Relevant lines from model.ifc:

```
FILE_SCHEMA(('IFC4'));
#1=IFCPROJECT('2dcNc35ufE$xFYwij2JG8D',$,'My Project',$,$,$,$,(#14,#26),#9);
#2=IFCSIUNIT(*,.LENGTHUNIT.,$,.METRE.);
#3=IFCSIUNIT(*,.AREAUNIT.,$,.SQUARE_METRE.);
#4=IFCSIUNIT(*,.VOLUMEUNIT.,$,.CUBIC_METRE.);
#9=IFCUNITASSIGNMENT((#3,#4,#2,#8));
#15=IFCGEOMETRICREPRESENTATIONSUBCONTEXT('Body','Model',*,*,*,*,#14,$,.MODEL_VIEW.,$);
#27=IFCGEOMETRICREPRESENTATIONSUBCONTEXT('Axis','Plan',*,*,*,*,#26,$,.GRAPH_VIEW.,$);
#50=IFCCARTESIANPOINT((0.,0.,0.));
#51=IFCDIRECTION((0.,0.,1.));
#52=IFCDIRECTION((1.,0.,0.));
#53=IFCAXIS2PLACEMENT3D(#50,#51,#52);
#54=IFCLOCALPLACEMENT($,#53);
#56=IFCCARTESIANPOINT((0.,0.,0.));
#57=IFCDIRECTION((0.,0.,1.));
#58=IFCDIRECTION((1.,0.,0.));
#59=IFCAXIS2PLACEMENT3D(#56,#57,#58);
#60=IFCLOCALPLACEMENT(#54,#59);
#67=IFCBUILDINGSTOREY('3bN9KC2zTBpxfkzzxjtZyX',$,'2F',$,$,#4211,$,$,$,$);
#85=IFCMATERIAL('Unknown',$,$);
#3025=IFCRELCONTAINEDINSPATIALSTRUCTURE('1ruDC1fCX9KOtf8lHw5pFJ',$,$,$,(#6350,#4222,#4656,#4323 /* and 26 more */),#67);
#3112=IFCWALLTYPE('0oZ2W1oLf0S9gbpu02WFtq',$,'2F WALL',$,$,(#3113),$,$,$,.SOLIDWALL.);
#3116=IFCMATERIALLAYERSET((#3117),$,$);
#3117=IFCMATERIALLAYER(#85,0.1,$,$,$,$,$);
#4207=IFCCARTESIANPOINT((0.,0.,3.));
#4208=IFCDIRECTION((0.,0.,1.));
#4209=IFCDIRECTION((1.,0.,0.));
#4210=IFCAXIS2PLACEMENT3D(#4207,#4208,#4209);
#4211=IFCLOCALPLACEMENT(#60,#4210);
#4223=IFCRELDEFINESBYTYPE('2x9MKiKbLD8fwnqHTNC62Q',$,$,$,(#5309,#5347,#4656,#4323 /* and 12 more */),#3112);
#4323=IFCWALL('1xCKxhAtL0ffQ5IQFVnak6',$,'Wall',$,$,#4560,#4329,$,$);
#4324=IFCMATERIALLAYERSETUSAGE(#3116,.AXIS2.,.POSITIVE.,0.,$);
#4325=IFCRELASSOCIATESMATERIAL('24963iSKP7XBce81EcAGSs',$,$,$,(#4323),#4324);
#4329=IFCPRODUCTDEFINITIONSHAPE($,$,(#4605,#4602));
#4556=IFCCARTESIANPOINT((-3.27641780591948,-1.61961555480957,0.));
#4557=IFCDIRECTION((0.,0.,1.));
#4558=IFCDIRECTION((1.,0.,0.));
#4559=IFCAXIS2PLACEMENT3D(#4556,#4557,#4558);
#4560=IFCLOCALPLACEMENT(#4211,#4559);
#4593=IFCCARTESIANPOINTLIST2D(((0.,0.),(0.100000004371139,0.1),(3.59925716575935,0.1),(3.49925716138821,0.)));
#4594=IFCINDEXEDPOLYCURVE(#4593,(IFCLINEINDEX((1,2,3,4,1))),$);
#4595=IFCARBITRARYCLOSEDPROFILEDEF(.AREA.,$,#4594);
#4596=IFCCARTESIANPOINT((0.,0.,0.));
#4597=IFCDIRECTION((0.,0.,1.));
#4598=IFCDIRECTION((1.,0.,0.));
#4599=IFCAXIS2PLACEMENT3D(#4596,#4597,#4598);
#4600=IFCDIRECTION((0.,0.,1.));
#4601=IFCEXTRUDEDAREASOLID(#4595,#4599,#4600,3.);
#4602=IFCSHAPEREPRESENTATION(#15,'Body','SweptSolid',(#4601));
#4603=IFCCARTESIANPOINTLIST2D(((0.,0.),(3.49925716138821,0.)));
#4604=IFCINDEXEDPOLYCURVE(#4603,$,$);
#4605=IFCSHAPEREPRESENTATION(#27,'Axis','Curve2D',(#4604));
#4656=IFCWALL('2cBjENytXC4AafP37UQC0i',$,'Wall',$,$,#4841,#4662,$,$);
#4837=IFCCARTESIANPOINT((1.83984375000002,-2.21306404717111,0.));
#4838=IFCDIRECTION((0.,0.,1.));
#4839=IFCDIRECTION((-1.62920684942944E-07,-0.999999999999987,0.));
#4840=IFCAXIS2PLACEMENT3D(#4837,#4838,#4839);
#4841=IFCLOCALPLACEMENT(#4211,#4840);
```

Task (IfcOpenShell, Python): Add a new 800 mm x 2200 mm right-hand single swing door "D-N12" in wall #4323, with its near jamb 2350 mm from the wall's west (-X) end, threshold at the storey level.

```python
import numpy as np
import ifcopenshell
import ifcopenshell.api.feature
import ifcopenshell.api.geometry
import ifcopenshell.api.root
import ifcopenshell.api.spatial
import ifcopenshell.geom
import ifcopenshell.util.element
import ifcopenshell.util.placement
import ifcopenshell.util.representation
import ifcopenshell.util.shape
import ifcopenshell.util.unit

model = ifcopenshell.open("model.ifc")
unit_scale = ifcopenshell.util.unit.calculate_unit_scale(model)
settings = ifcopenshell.geom.settings()


def volume(element):
    """Net volume in cubic metres, openings subtracted."""
    shape = ifcopenshell.geom.create_shape(settings, element)
    return ifcopenshell.util.shape.get_volume(shape.geometry)


wall = model.by_guid("1xCKxhAtL0ffQ5IQFVnak6")
storey = ifcopenshell.util.element.get_container(wall, ifc_class="IfcBuildingStorey")
context = ifcopenshell.util.representation.get_context(model, "Model", "Body", "MODEL_VIEW")
before = volume(wall)

width, height, from_end, sill = 0.8, 2.2, 2.35, 0.0  # metres

# The wall runs along its own X axis, and the end named is its -X end.
wall_shape = ifcopenshell.geom.create_shape(settings, wall)
x, y, z = ifcopenshell.util.shape.get_vertices(wall_shape.geometry).T
start = x.min() + from_end
face, thickness = float(y.min()), float(y.max() - y.min())
wall_matrix = ifcopenshell.util.placement.get_local_placement(wall.ObjectPlacement)
level = ifcopenshell.util.placement.get_local_placement(storey.ObjectPlacement)[2, 3]


def in_wall(x, y):
    """Placement at x, y metres in the wall's axes, at sill height."""
    matrix = wall_matrix.copy()
    matrix[:, 3] = wall_matrix @ np.array([x / unit_scale, y / unit_scale, 0.0, 1.0])
    matrix[2, 3] = level + sill / unit_scale
    return matrix


# Opening: a box that overshoots both wall faces by 50 mm.
opening = ifcopenshell.api.root.create_entity(model, ifc_class="IfcOpeningElement", predefined_type="OPENING")
box = ifcopenshell.api.geometry.add_wall_representation(
    model, context=context, length=width, height=height, thickness=thickness + 0.1
)
ifcopenshell.api.geometry.assign_representation(model, product=opening, representation=box)
ifcopenshell.api.geometry.edit_object_placement(model, product=opening, matrix=in_wall(start, face - 0.05), is_si=False)
ifcopenshell.api.feature.add_feature(model, feature=opening, element=wall)

door = ifcopenshell.api.root.create_entity(model, ifc_class="IfcDoor", name="D-N12", predefined_type="DOOR")
door.OverallWidth, door.OverallHeight = width / unit_scale, height / unit_scale
door.OperationType = "SINGLE_SWING_RIGHT"
body = ifcopenshell.api.geometry.add_door_representation(
    model,
    context=context,
    overall_width=door.OverallWidth,
    overall_height=door.OverallHeight,
    operation_type="SINGLE_SWING_RIGHT",
    lining_properties={"LiningDepth": thickness / unit_scale, "ThresholdDepth": thickness / unit_scale},
)
ifcopenshell.api.geometry.assign_representation(model, product=door, representation=body)
ifcopenshell.api.spatial.assign_container(model, products=[door], relating_structure=storey)
ifcopenshell.api.feature.add_filling(model, opening=opening, element=door)

# The lining spans the wall, so the door starts at the wall face.
ifcopenshell.api.geometry.edit_object_placement(model, product=door, matrix=in_wall(start, face), is_si=False)

after = volume(wall)

print(f"wall volume {before:.3f} -> {after:.3f} m3")

model.write("model_updated.ifc")
```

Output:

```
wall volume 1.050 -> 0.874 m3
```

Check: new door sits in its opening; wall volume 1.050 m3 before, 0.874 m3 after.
